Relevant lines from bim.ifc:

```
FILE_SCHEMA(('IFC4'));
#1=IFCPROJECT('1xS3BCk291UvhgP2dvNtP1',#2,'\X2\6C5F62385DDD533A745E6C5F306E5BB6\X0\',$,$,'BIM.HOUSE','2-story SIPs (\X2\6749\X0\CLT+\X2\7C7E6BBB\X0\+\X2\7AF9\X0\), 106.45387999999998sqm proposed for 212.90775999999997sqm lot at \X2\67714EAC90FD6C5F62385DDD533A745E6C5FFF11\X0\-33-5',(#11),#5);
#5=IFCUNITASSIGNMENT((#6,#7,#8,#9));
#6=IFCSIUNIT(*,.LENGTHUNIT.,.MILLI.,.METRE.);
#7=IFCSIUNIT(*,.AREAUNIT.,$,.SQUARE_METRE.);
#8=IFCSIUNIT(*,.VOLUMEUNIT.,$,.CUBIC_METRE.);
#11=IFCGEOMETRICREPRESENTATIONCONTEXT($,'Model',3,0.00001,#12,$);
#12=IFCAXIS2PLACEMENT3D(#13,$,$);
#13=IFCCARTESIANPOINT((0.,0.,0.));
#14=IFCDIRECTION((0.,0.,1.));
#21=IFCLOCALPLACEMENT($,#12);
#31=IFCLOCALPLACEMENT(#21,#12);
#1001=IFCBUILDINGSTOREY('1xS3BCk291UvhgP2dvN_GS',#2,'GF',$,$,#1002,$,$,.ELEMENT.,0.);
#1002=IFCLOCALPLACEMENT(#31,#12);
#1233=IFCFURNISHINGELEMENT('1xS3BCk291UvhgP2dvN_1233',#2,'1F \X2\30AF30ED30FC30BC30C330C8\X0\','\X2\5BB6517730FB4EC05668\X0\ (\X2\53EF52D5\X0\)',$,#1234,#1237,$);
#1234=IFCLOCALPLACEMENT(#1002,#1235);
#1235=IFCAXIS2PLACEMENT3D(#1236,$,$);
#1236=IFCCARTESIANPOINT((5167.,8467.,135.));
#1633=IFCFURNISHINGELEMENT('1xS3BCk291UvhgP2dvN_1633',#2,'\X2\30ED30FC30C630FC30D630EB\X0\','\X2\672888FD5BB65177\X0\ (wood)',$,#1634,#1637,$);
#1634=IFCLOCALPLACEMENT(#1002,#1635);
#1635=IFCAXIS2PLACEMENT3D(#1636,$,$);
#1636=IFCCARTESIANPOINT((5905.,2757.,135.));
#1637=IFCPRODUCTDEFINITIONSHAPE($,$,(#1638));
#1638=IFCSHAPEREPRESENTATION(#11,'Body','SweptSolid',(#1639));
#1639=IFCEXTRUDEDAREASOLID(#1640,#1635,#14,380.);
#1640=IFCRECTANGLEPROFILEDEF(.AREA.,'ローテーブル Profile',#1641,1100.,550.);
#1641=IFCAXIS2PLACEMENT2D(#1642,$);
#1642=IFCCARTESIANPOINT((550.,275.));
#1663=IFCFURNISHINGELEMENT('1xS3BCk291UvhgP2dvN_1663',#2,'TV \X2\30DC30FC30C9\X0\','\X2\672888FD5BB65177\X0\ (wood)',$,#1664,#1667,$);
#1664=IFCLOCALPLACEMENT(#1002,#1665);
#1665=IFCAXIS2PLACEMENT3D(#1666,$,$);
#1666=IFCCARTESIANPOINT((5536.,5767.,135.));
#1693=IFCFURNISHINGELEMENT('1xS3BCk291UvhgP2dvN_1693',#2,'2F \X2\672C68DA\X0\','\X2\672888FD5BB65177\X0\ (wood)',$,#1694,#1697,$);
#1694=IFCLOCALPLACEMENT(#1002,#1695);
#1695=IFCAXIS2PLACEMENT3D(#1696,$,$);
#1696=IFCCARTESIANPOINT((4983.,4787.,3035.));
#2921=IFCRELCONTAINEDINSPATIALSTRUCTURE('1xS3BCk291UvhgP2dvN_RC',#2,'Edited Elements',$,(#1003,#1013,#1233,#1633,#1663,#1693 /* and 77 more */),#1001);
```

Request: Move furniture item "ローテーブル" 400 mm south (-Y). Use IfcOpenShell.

```python
import ifcopenshell
import ifcopenshell.api.geometry
import ifcopenshell.util.placement

model = ifcopenshell.open("bim.ifc")

item = model.by_guid("1xS3BCk291UvhgP2dvN_1633")
matrix = ifcopenshell.util.placement.get_local_placement(item.ObjectPlacement)
matrix[1, 3] -= 400.0
ifcopenshell.api.geometry.edit_object_placement(model, product=item, matrix=matrix, is_si=False)

print(ifcopenshell.util.placement.get_local_placement(item.ObjectPlacement).round(3) + 0.0)

model.write("bim_updated.ifc")
```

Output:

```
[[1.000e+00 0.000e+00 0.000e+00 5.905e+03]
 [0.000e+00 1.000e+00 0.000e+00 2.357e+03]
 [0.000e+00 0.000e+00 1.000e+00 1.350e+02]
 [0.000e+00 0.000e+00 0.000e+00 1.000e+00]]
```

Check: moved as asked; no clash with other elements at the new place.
